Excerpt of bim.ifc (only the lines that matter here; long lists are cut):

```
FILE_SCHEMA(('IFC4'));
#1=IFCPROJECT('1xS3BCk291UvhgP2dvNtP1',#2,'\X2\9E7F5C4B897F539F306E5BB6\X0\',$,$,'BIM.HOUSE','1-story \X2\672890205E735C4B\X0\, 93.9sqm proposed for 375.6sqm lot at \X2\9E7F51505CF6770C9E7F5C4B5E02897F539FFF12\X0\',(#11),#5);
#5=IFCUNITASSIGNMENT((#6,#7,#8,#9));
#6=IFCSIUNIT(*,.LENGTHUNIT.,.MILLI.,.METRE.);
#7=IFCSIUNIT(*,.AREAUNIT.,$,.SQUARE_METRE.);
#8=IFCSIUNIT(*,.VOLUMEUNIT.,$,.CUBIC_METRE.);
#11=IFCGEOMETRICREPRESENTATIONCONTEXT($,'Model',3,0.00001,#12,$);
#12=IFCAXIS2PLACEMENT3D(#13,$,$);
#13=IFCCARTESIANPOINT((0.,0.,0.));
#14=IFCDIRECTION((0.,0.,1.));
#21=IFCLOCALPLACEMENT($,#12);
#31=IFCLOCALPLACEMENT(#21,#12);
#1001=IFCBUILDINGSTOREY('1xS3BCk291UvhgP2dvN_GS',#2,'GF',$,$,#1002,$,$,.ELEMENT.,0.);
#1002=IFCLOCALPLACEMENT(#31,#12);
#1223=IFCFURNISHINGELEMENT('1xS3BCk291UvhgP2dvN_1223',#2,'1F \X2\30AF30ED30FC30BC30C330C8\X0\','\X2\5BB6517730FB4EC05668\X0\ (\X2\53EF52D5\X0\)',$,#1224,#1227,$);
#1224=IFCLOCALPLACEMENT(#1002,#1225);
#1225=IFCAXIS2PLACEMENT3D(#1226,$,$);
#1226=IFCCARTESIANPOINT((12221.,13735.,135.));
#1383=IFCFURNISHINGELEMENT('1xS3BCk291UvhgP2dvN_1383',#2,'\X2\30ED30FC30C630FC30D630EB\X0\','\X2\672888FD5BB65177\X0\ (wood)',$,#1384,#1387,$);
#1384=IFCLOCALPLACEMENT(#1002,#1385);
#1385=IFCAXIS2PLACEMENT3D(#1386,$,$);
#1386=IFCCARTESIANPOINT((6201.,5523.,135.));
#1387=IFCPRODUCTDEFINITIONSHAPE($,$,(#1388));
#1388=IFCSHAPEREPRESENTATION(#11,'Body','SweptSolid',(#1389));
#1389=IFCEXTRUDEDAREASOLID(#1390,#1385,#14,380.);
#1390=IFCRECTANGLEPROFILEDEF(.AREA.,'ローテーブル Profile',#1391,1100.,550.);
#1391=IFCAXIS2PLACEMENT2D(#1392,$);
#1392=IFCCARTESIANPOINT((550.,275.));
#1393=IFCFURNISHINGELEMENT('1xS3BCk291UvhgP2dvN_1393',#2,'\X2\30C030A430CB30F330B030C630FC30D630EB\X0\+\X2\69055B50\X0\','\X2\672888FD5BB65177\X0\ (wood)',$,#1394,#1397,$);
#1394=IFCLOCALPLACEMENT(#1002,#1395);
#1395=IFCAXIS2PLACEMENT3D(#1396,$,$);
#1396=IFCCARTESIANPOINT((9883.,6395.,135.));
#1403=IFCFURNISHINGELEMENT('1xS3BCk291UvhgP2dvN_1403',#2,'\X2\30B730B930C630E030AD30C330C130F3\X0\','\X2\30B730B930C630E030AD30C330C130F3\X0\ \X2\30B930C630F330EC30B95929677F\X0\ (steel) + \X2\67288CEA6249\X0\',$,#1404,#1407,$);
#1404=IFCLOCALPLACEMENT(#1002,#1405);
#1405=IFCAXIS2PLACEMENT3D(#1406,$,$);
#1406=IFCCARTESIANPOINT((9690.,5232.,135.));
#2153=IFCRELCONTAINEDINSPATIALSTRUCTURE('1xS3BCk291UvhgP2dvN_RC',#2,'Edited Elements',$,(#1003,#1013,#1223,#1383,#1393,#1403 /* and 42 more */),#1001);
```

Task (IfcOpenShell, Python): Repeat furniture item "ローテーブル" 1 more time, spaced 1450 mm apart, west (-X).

```python
import numpy as np
import ifcopenshell
import ifcopenshell.api.geometry
import ifcopenshell.api.root
import ifcopenshell.util.element
import ifcopenshell.util.placement
import ifcopenshell.util.unit

model = ifcopenshell.open("bim.ifc")
unit_scale = ifcopenshell.util.unit.calculate_unit_scale(model)


def reuse_history(source, copy):
    """copy_class also copies each property set's owner history, people and application; keep the originals."""
    for rel in copy.IsDefinedBy:
        if rel.is_a("IfcRelDefinesByProperties") and (history := rel.RelatingPropertyDefinition.OwnerHistory):
            rel.RelatingPropertyDefinition.OwnerHistory = source.OwnerHistory
            ifcopenshell.util.element.remove_deep2(model, history)


source = model.by_guid("1xS3BCk291UvhgP2dvN_1383")
base = ifcopenshell.util.placement.get_local_placement(source.ObjectPlacement)
step = np.array([-1.0, 0.0, 0.0]) * 1.45 / unit_scale

for i in range(1, 2):
    copy = ifcopenshell.api.root.copy_class(model, product=source)
    copy.Representation = ifcopenshell.util.element.copy_deep(
        model, source.Representation, exclude=["IfcGeometricRepresentationContext", "IfcRepresentationMap"]
    )
    reuse_history(source, copy)
    matrix = base.copy()
    matrix[:3, 3] += i * step
    print("added at", matrix[:3, 3].round(3) + 0.0)
    ifcopenshell.api.geometry.edit_object_placement(model, product=copy, matrix=matrix, is_si=False)

model.write("bim-out.ifc")
```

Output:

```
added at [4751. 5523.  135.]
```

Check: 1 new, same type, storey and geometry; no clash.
